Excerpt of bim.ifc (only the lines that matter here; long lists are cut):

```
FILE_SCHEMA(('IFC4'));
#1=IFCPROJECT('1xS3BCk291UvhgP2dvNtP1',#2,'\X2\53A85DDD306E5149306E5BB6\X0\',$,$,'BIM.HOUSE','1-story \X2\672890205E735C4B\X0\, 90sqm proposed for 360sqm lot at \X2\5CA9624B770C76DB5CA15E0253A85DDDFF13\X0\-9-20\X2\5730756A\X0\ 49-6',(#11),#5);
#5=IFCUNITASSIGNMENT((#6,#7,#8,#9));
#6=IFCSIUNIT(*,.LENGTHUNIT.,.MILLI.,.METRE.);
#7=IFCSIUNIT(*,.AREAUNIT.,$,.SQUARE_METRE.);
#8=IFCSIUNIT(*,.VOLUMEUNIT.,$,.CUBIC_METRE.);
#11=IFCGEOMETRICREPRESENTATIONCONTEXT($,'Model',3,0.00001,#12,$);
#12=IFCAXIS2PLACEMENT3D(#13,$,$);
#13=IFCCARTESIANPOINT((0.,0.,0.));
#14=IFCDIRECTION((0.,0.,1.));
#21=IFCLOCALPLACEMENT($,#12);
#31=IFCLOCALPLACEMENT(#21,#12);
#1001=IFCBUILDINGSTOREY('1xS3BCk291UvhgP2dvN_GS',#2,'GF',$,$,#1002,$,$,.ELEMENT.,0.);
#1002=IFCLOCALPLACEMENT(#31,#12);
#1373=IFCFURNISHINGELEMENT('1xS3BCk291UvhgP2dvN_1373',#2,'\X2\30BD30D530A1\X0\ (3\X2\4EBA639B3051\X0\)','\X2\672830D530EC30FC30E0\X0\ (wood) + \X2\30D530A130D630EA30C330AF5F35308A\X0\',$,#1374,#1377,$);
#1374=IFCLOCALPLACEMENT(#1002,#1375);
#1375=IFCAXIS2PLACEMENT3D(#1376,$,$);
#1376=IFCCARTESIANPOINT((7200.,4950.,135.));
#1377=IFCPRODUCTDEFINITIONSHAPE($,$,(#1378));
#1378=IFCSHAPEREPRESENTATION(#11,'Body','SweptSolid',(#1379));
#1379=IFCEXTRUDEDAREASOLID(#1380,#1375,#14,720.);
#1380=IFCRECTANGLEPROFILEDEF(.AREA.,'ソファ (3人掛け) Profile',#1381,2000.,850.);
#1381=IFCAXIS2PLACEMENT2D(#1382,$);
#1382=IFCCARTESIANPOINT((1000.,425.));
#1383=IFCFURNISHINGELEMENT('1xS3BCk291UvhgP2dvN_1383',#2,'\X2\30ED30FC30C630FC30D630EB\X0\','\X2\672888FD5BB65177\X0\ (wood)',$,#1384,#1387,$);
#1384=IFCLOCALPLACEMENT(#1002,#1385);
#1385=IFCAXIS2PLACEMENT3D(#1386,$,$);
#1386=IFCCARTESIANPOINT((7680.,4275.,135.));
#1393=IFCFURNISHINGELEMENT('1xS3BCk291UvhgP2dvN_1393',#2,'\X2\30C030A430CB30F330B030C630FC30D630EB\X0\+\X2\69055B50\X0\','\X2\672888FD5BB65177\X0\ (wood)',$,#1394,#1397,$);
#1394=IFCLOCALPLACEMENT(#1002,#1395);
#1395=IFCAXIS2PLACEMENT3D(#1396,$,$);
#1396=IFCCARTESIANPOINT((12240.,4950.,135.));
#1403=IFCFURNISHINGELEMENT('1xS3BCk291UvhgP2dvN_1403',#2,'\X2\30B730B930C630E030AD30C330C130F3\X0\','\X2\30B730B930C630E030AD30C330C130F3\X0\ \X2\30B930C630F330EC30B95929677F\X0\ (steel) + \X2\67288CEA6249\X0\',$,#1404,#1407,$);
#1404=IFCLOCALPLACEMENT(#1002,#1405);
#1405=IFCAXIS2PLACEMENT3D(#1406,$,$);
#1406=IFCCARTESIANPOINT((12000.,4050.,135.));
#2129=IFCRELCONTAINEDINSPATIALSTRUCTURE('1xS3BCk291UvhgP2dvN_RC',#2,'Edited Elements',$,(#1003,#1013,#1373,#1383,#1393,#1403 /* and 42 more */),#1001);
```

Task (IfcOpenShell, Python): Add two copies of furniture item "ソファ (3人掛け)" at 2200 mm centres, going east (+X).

```python
import numpy as np
import ifcopenshell
import ifcopenshell.api.geometry
import ifcopenshell.api.root
import ifcopenshell.util.element
import ifcopenshell.util.placement

model = ifcopenshell.open("bim.ifc")


def reuse_history(source, copy):
    """copy_class also copies each property set's owner history, people and application; keep the originals."""
    for rel in copy.IsDefinedBy:
        if rel.is_a("IfcRelDefinesByProperties") and (history := rel.RelatingPropertyDefinition.OwnerHistory):
            rel.RelatingPropertyDefinition.OwnerHistory = source.OwnerHistory
            ifcopenshell.util.element.remove_deep2(model, history)


source = model.by_id(1373)
base = ifcopenshell.util.placement.get_local_placement(source.ObjectPlacement)
step = np.array([1.0, 0.0, 0.0]) * 2200.0

for i in range(1, 3):
    copy = ifcopenshell.api.root.copy_class(model, product=source)
    copy.Representation = ifcopenshell.util.element.copy_deep(
        model, source.Representation, exclude=["IfcGeometricRepresentationContext", "IfcRepresentationMap"]
    )
    reuse_history(source, copy)
    matrix = base.copy()
    matrix[:3, 3] += i * step
    print("added at", matrix[:3, 3].round(3) + 0.0)
    ifcopenshell.api.geometry.edit_object_placement(model, product=copy, matrix=matrix, is_si=False)

model.write("bim_rev.ifc")
```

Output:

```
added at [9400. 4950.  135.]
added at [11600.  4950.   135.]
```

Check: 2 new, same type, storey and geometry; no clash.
